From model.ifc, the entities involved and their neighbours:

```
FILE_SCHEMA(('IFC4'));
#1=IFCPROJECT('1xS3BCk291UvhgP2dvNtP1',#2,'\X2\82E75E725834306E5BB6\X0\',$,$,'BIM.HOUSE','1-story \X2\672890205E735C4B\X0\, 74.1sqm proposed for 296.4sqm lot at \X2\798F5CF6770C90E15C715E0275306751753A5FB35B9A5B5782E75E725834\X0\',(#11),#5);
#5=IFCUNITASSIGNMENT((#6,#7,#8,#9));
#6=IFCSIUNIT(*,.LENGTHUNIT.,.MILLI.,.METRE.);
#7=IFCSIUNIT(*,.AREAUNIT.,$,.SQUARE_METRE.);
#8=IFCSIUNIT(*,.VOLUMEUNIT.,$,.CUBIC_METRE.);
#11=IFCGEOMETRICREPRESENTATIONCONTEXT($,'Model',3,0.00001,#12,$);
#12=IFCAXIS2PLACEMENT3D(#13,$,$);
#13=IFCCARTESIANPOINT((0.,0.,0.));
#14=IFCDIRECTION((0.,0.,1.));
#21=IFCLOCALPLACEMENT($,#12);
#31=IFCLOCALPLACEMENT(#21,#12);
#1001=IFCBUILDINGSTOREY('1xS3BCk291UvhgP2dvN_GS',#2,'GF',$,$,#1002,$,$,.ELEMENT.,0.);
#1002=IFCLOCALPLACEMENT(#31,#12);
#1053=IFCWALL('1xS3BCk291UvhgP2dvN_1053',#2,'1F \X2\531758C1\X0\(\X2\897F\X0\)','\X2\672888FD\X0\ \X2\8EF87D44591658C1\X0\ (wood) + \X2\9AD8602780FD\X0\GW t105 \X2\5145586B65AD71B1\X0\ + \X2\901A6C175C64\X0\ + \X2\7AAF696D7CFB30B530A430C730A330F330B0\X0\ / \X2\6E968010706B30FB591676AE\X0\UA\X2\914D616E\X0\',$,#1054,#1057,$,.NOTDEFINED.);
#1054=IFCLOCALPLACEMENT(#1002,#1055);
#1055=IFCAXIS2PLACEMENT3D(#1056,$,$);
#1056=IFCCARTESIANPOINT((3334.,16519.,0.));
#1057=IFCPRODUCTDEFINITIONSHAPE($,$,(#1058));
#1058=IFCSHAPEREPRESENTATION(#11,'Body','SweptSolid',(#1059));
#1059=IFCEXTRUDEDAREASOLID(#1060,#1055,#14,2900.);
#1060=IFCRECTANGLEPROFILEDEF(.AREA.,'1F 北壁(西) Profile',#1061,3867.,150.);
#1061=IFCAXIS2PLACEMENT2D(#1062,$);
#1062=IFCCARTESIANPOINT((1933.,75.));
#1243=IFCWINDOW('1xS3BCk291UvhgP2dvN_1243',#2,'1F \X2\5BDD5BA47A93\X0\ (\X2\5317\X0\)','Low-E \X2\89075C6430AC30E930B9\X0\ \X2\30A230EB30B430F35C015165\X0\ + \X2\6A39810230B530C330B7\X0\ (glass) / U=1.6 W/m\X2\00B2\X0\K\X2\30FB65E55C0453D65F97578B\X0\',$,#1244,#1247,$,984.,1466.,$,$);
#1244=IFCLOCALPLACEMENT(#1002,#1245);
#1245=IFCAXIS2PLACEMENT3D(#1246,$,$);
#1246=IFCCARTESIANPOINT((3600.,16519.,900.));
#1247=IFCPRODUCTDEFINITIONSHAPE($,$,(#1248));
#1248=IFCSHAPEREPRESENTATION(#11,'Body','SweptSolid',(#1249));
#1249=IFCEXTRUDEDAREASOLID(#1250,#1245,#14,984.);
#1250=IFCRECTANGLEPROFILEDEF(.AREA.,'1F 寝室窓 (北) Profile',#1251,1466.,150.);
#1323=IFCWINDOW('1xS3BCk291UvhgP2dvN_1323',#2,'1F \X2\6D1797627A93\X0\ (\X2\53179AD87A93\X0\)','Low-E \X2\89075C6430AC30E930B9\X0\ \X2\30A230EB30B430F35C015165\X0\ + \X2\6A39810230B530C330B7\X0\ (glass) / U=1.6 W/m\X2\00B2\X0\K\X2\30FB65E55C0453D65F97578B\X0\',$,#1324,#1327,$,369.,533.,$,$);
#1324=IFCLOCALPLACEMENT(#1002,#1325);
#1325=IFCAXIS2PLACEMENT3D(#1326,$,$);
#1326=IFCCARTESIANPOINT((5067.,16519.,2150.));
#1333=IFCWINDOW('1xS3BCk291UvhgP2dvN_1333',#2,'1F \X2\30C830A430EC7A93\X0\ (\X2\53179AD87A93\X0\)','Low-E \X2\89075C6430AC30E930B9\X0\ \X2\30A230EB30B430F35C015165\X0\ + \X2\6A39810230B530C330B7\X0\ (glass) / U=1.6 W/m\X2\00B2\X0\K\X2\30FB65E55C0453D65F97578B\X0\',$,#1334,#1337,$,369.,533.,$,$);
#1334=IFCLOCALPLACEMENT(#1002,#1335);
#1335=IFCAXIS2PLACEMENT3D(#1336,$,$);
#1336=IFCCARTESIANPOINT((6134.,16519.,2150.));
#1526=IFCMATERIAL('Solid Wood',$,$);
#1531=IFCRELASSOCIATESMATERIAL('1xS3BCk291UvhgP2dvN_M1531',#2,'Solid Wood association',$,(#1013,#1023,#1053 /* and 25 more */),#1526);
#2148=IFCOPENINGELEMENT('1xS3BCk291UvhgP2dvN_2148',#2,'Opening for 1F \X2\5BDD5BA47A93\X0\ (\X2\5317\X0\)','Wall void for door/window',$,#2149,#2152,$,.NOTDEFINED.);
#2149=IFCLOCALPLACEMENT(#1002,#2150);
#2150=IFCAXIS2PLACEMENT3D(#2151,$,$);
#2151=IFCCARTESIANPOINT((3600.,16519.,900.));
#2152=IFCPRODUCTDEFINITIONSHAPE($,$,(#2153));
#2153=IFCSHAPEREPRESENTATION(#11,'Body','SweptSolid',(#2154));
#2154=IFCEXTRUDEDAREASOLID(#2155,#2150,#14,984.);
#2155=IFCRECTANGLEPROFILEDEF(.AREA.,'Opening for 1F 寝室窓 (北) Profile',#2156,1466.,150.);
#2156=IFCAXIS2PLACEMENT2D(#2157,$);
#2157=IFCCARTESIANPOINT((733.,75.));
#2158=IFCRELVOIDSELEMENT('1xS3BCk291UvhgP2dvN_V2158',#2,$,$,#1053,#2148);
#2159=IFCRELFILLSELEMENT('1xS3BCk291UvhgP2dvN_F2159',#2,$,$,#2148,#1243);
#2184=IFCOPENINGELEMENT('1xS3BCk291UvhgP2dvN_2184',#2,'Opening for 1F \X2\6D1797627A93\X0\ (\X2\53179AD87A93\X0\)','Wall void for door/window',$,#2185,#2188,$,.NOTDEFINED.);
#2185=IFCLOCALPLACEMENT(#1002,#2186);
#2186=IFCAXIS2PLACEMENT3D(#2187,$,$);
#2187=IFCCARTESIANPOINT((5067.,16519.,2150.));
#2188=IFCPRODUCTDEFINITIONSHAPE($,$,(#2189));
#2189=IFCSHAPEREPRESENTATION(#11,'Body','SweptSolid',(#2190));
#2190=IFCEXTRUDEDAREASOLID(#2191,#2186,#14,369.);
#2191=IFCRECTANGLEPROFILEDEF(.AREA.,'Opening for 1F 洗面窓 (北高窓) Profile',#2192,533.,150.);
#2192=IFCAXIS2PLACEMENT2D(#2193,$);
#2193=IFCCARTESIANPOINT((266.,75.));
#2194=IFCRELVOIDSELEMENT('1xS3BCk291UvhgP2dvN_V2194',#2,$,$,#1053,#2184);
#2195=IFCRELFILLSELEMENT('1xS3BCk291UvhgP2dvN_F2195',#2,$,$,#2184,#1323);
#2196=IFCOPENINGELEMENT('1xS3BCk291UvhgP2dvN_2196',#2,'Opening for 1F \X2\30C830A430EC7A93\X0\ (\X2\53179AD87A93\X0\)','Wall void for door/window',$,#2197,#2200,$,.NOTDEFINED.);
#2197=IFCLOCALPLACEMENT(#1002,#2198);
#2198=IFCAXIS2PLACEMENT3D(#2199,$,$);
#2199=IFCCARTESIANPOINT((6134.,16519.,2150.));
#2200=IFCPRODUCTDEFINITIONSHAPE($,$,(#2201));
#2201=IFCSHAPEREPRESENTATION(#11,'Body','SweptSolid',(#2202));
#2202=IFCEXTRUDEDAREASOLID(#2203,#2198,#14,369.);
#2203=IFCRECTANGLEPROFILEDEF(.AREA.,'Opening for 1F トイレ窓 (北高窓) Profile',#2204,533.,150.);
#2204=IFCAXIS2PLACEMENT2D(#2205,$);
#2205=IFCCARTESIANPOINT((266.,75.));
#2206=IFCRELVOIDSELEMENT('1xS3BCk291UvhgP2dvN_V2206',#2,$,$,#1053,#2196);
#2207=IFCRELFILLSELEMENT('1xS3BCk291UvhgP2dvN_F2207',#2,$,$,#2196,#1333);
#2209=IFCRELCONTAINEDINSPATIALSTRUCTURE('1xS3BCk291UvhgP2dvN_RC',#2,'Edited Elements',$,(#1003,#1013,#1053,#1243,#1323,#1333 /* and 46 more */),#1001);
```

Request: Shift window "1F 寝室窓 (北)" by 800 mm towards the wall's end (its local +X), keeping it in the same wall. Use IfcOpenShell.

```python
import ifcopenshell
import ifcopenshell.api.geometry
import ifcopenshell.util.placement

model = ifcopenshell.open("model.ifc")

window = model.by_id(1243)
opening = window.FillsVoids[0].RelatingOpeningElement
wall = opening.VoidsElements[0].RelatingBuildingElement

wall_matrix = ifcopenshell.util.placement.get_local_placement(wall.ObjectPlacement)
shift = wall_matrix[:3, 0] * 800.0
before = ifcopenshell.util.placement.get_local_placement(window.ObjectPlacement)[:3, 3].copy()

# The window is not placed relative to its opening, so move both.
for product in (opening, window):
    matrix = ifcopenshell.util.placement.get_local_placement(product.ObjectPlacement)
    matrix[:3, 3] += shift
    ifcopenshell.api.geometry.edit_object_placement(model, product=product, matrix=matrix, is_si=False)

after = ifcopenshell.util.placement.get_local_placement(window.ObjectPlacement)[:3, 3]
print("window moved by", (after - before).round(3) + 0.0)

model.write("model_v2.ifc")
```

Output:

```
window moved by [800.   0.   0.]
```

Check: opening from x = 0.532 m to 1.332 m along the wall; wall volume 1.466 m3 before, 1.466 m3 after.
